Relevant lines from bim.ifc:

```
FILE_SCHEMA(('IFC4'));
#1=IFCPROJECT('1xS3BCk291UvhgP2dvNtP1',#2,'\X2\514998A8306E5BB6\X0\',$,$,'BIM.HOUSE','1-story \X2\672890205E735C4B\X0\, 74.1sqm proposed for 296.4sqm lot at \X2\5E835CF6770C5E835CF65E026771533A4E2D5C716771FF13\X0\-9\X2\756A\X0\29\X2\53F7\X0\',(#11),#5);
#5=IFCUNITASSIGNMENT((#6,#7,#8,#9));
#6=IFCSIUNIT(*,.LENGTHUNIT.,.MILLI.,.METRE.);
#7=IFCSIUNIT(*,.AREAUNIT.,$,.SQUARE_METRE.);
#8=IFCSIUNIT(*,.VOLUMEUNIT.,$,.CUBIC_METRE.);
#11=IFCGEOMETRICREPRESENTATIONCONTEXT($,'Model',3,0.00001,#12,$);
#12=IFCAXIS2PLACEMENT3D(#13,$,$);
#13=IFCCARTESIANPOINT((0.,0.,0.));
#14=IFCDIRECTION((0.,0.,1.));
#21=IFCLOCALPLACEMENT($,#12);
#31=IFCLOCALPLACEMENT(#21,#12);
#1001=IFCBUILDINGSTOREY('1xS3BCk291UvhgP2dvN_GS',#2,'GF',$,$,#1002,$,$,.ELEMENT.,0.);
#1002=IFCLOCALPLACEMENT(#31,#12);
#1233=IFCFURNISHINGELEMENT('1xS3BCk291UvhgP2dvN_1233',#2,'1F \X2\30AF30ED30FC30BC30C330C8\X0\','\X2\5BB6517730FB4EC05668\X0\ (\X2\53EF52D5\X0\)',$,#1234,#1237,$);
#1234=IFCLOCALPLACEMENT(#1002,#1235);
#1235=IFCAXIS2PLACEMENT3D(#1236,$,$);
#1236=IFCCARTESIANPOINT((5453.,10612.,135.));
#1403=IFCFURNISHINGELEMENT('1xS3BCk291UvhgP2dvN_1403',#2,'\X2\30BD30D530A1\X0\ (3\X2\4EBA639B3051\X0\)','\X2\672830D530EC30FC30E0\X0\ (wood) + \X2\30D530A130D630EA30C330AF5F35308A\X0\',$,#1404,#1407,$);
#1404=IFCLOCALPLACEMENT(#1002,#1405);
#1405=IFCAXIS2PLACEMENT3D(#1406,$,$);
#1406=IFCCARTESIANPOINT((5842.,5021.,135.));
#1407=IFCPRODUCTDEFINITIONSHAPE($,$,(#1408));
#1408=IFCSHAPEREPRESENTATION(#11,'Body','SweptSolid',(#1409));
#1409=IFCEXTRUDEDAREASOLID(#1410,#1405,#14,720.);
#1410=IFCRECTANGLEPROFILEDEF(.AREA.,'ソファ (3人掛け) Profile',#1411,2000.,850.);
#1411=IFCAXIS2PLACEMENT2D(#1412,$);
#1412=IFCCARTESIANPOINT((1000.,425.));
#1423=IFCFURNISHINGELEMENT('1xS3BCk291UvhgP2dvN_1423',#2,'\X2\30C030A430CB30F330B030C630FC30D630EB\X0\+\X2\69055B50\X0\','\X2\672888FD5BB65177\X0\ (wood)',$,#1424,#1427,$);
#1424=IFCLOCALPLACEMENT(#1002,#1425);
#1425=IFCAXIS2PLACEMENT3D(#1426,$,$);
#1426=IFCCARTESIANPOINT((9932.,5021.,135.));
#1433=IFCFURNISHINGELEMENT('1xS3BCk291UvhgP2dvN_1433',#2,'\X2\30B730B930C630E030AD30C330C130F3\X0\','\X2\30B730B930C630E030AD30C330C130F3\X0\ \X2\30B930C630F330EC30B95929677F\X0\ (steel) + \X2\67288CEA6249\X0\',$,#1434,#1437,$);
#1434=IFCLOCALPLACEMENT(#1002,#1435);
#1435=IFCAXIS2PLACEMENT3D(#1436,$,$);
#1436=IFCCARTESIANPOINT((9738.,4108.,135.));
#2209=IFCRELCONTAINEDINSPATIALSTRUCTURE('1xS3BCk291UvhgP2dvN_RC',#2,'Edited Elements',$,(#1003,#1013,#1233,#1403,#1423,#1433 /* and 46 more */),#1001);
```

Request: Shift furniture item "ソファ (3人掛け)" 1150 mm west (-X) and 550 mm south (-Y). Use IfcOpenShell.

```python
import ifcopenshell
import ifcopenshell.api.geometry
import ifcopenshell.util.placement
import ifcopenshell.util.unit

model = ifcopenshell.open("bim.ifc")
unit_scale = ifcopenshell.util.unit.calculate_unit_scale(model)

item = model.by_guid("1xS3BCk291UvhgP2dvN_1403")
matrix = ifcopenshell.util.placement.get_local_placement(item.ObjectPlacement)
matrix[0, 3] -= 1.15 / unit_scale
matrix[1, 3] -= 0.55 / unit_scale
ifcopenshell.api.geometry.edit_object_placement(model, product=item, matrix=matrix, is_si=False)

print(ifcopenshell.util.placement.get_local_placement(item.ObjectPlacement).round(3) + 0.0)

model.write("bim_rev.ifc")
```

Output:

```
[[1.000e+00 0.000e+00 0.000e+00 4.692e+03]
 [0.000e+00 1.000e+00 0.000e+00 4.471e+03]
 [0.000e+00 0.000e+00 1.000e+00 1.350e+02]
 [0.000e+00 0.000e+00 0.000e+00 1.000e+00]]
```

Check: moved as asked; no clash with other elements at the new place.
